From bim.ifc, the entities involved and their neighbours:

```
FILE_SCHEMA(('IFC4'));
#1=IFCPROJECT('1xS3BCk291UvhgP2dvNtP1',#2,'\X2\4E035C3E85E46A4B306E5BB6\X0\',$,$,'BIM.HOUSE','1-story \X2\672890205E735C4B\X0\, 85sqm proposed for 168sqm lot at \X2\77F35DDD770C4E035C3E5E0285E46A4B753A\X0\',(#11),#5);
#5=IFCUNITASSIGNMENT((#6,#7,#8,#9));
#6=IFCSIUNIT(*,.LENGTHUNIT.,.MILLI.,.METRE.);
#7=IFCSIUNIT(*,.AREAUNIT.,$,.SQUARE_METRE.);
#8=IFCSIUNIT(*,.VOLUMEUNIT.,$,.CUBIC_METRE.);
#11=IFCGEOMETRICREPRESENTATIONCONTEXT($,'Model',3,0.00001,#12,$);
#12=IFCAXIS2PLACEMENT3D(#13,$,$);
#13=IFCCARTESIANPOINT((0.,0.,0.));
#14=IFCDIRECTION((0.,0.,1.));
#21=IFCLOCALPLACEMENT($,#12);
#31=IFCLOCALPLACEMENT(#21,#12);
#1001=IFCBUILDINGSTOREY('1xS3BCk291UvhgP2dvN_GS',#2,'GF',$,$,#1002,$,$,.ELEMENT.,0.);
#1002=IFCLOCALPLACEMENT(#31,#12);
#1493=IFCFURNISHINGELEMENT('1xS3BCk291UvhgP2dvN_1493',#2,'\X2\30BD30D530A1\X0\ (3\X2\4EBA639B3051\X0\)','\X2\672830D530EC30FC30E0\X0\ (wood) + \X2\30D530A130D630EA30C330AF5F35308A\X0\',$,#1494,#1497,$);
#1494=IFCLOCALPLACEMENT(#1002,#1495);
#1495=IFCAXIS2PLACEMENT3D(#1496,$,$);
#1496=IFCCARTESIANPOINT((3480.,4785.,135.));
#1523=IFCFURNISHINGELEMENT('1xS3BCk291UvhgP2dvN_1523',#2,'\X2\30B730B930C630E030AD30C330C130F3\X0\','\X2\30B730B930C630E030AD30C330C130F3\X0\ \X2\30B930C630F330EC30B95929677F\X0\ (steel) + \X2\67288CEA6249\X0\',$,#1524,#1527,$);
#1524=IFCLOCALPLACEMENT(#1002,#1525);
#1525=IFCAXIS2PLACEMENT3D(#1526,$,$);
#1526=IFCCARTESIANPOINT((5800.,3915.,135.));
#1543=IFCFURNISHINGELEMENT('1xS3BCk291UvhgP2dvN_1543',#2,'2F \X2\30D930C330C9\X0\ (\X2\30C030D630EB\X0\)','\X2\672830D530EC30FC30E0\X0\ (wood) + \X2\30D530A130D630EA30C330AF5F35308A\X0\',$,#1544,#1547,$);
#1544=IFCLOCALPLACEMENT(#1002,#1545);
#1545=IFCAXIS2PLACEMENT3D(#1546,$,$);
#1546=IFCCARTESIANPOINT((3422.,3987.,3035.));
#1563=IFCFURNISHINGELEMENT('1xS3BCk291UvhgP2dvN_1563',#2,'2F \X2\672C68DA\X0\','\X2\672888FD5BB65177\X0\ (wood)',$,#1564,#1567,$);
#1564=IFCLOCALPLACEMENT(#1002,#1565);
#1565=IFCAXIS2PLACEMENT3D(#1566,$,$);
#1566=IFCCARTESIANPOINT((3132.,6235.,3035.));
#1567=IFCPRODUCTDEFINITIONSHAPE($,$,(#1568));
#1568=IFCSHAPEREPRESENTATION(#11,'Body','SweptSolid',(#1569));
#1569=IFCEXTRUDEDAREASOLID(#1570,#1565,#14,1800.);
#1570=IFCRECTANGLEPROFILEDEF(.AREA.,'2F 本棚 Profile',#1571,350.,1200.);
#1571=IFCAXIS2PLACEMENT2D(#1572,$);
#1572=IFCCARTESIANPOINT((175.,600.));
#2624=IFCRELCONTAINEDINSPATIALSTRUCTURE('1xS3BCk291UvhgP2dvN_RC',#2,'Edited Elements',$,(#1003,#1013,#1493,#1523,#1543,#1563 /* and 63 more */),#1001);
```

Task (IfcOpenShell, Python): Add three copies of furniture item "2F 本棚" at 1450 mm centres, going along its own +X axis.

```python
import ifcopenshell
import ifcopenshell.api.geometry
import ifcopenshell.api.root
import ifcopenshell.util.element
import ifcopenshell.util.placement
import ifcopenshell.util.unit

model = ifcopenshell.open("bim.ifc")
unit_scale = ifcopenshell.util.unit.calculate_unit_scale(model)


def reuse_history(source, copy):
    """copy_class also copies each property set's owner history, people and application; keep the originals."""
    for rel in copy.IsDefinedBy:
        if rel.is_a("IfcRelDefinesByProperties") and (history := rel.RelatingPropertyDefinition.OwnerHistory):
            rel.RelatingPropertyDefinition.OwnerHistory = source.OwnerHistory
            ifcopenshell.util.element.remove_deep2(model, history)


source = model.by_guid("1xS3BCk291UvhgP2dvN_1563")
base = ifcopenshell.util.placement.get_local_placement(source.ObjectPlacement)
step = base[:3, 0] * 1.45 / unit_scale

for i in range(1, 4):
    copy = ifcopenshell.api.root.copy_class(model, product=source)
    copy.Representation = ifcopenshell.util.element.copy_deep(
        model, source.Representation, exclude=["IfcGeometricRepresentationContext", "IfcRepresentationMap"]
    )
    reuse_history(source, copy)
    matrix = base.copy()
    matrix[:3, 3] += i * step
    print("added at", matrix[:3, 3].round(3) + 0.0)
    ifcopenshell.api.geometry.edit_object_placement(model, product=copy, matrix=matrix, is_si=False)

model.write("bim_v2.ifc")
```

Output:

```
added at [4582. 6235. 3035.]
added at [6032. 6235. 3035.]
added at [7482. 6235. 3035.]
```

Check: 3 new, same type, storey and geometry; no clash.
